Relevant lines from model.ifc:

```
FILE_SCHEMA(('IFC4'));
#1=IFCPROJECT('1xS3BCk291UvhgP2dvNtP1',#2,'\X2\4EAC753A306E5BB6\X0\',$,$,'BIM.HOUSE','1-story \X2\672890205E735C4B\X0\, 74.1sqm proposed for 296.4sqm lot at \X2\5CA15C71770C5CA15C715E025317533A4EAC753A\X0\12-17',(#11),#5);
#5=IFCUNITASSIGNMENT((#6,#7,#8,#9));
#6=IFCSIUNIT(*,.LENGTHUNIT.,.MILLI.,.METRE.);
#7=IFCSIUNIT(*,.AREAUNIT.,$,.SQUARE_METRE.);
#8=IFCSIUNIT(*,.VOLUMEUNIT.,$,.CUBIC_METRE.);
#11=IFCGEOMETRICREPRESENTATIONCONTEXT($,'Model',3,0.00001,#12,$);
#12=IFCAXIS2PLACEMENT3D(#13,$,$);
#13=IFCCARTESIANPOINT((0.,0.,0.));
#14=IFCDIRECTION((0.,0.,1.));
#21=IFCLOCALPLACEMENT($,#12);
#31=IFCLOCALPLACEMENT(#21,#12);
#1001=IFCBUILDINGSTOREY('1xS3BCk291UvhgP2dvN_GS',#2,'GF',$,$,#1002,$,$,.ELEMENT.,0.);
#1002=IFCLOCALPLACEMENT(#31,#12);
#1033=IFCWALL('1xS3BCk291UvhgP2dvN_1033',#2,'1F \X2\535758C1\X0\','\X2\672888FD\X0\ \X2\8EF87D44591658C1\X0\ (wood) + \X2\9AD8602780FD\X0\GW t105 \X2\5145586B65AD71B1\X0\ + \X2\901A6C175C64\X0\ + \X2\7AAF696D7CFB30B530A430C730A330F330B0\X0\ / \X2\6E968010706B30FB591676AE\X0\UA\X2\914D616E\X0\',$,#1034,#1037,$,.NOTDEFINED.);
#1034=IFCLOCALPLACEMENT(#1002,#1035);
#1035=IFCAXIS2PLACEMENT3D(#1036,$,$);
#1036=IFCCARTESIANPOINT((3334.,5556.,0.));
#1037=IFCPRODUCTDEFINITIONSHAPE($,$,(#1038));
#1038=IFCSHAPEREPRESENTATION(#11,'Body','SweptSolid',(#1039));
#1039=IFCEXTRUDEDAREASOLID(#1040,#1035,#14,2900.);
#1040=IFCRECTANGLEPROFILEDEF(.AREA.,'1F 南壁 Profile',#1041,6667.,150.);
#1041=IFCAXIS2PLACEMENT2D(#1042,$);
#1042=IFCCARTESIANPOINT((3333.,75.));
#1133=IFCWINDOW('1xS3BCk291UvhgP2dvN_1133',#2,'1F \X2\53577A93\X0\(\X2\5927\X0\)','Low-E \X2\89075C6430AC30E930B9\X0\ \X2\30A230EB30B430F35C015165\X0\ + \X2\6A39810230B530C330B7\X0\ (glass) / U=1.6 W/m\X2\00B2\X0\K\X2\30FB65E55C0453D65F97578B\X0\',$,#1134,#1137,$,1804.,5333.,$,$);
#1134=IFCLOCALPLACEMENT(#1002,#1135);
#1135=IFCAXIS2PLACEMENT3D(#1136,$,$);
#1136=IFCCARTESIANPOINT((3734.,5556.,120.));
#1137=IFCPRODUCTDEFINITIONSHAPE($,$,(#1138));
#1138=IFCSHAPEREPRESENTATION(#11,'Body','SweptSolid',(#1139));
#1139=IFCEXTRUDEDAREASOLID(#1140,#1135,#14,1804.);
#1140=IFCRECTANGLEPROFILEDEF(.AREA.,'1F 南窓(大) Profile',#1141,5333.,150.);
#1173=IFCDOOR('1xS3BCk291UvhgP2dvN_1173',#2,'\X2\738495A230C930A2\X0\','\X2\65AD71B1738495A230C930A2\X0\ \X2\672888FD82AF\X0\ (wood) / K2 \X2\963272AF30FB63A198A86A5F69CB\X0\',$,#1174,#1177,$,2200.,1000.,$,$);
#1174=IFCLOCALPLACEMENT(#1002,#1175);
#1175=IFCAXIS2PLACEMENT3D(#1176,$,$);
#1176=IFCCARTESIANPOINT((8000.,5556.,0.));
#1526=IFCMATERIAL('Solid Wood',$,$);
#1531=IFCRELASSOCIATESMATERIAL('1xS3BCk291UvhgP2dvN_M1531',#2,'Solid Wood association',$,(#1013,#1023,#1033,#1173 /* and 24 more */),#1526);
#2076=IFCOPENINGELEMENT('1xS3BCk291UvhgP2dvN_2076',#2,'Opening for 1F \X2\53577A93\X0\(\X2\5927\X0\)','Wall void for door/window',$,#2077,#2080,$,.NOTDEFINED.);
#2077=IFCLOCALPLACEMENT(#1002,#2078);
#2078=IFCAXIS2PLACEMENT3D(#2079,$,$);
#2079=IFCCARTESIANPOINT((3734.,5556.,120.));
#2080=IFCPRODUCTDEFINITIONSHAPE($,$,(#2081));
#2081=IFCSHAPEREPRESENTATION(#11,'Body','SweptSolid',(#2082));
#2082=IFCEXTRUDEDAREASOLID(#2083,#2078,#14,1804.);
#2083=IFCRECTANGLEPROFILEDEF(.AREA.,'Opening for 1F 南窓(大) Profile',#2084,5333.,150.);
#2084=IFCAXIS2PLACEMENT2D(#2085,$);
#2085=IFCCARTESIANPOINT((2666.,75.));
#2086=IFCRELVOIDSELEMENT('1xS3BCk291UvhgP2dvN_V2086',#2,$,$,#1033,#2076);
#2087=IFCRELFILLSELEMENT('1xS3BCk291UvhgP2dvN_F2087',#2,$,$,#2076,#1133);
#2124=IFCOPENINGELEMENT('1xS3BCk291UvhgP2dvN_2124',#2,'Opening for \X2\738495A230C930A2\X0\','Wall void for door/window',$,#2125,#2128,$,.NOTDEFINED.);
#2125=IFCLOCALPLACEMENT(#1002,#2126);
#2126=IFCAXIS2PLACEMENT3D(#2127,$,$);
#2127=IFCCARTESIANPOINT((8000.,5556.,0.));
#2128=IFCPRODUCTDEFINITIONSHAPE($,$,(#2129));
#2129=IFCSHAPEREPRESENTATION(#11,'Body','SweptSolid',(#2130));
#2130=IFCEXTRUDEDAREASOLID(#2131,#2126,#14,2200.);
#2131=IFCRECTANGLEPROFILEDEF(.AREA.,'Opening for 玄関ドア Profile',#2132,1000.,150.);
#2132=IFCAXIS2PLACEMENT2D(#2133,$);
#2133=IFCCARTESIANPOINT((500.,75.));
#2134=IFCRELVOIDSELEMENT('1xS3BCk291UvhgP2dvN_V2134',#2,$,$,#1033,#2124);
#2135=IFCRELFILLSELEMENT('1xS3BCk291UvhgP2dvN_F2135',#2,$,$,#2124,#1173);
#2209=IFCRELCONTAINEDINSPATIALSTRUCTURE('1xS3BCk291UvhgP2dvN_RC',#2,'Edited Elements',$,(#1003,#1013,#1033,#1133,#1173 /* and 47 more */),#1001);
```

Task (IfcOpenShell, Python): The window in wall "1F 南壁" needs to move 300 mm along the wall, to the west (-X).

```python
import ifcopenshell
import ifcopenshell.api.geometry
import ifcopenshell.util.placement
import ifcopenshell.util.unit

model = ifcopenshell.open("model.ifc")
unit_scale = ifcopenshell.util.unit.calculate_unit_scale(model)

window = model.by_guid("1xS3BCk291UvhgP2dvN_1133")
opening = window.FillsVoids[0].RelatingOpeningElement
wall = opening.VoidsElements[0].RelatingBuildingElement

wall_matrix = ifcopenshell.util.placement.get_local_placement(wall.ObjectPlacement)
shift = wall_matrix[:3, 0] * -0.3 / unit_scale
before = ifcopenshell.util.placement.get_local_placement(window.ObjectPlacement)[:3, 3].copy()

# The window is not placed relative to its opening, so move both.
for product in (opening, window):
    matrix = ifcopenshell.util.placement.get_local_placement(product.ObjectPlacement)
    matrix[:3, 3] += shift
    ifcopenshell.api.geometry.edit_object_placement(model, product=product, matrix=matrix, is_si=False)

after = ifcopenshell.util.placement.get_local_placement(window.ObjectPlacement)[:3, 3]
print("window moved by", (after - before).round(3) + 0.0)

model.write("model_v2.ifc")
```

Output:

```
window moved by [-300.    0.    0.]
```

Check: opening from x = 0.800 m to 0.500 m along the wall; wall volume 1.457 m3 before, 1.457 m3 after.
